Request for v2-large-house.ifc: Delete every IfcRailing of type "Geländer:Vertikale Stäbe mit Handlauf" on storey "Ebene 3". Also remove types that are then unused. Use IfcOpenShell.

First a look at what the model holds.

```python
import ifcopenshell
import ifcopenshell.util.element

model = ifcopenshell.open("v2-large-house.ifc")
print(model.schema)
storey = next(s for s in model.by_type("IfcBuildingStorey") if s.Name == "Ebene 3")
railings = [e for e in ifcopenshell.util.element.get_decomposition(storey) if e.is_a("IfcRailing")]
seen = {}
for e in railings:
    element_type = ifcopenshell.util.element.get_type(e)
    name = element_type.Name if element_type not in (None, e) else None
    seen[name] = seen.get(name, 0) + 1
for name, count in sorted(seen.items(), key=str):
    print(count, "x", name)
```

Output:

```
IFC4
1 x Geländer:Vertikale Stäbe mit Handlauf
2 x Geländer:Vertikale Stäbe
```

```python
import ifcopenshell
import ifcopenshell.api.root
import ifcopenshell.util.element

model = ifcopenshell.open("v2-large-house.ifc")

storey = next(s for s in model.by_type("IfcBuildingStorey") if s.Name == "Ebene 3")
railings = [e for e in ifcopenshell.util.element.get_decomposition(storey) if e.is_a("IfcRailing")]
targets = [e for e in railings if (t := ifcopenshell.util.element.get_type(e)) not in (None, e) and t.Name == "Geländer:Vertikale Stäbe mit Handlauf"]
types = {ifcopenshell.util.element.get_type(e) for e in targets} - {None, *targets}

for e in targets:
    ifcopenshell.api.root.remove_product(model, product=e)
print(len(targets), "removed")

unused = [t for t in types if not ifcopenshell.util.element.get_types(t)]
for t in unused:
    ifcopenshell.api.root.remove_product(model, product=t)
print(len(unused), "unused types removed")

model.write("v2-large-house_v2.ifc")
```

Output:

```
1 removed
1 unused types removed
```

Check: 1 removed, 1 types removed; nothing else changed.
